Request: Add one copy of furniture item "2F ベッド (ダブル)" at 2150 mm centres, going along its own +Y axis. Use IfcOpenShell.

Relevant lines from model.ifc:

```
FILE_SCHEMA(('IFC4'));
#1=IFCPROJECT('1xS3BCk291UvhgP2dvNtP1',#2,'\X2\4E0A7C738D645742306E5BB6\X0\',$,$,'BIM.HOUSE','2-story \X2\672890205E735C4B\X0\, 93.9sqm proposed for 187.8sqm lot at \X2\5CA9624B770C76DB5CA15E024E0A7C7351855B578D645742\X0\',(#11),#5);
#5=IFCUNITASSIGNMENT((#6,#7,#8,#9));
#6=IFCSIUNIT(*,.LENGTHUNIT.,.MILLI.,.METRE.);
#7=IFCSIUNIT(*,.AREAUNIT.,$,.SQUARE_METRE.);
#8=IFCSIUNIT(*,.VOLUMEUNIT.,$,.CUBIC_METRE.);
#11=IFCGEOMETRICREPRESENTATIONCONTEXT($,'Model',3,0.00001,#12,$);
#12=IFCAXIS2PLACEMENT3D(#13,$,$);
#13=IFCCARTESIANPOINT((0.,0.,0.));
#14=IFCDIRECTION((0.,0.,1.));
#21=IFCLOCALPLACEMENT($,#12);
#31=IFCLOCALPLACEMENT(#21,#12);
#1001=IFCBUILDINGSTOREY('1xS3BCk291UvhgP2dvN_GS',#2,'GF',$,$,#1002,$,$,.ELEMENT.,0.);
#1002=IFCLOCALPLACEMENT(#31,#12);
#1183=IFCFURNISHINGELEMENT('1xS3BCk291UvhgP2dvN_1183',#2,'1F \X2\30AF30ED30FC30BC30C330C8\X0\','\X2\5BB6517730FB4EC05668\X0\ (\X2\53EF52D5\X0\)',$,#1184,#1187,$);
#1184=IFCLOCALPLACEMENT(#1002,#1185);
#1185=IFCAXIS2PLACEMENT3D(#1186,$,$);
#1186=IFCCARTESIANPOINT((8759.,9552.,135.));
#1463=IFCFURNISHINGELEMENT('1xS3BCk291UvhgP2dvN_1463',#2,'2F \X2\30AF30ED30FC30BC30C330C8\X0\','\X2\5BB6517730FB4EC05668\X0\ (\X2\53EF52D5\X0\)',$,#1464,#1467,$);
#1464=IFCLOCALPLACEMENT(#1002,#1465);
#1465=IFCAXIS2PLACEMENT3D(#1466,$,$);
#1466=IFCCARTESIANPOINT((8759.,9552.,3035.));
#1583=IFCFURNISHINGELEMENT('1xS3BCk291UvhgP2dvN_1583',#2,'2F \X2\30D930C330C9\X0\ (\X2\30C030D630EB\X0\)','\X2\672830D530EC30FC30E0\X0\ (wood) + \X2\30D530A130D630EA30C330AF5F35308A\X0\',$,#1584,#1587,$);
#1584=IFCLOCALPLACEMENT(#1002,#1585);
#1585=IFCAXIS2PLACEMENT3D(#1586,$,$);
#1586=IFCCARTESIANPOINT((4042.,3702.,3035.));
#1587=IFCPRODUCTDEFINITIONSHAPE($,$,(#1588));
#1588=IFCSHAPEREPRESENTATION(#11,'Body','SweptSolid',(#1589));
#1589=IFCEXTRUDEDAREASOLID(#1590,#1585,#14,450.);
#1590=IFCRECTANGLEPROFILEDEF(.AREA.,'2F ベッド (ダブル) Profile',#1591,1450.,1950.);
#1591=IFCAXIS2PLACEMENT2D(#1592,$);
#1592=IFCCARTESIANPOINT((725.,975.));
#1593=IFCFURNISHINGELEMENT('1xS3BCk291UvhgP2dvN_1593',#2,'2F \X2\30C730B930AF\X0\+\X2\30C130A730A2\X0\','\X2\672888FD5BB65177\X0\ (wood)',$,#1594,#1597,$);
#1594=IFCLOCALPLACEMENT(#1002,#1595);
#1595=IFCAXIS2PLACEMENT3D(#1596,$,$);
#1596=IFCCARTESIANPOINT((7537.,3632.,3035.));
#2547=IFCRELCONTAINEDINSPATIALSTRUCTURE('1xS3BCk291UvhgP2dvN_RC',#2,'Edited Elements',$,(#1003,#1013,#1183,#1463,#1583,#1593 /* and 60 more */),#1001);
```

```python
import ifcopenshell
import ifcopenshell.api.geometry
import ifcopenshell.api.root
import ifcopenshell.util.element
import ifcopenshell.util.placement
import ifcopenshell.util.unit

model = ifcopenshell.open("model.ifc")
unit_scale = ifcopenshell.util.unit.calculate_unit_scale(model)


def reuse_history(source, copy):
    """copy_class also copies each property set's owner history, people and application; keep the originals."""
    for rel in copy.IsDefinedBy:
        if rel.is_a("IfcRelDefinesByProperties") and (history := rel.RelatingPropertyDefinition.OwnerHistory):
            rel.RelatingPropertyDefinition.OwnerHistory = source.OwnerHistory
            ifcopenshell.util.element.remove_deep2(model, history)


source = model.by_id(1583)
base = ifcopenshell.util.placement.get_local_placement(source.ObjectPlacement)
step = base[:3, 1] * 2.15 / unit_scale

for i in range(1, 2):
    copy = ifcopenshell.api.root.copy_class(model, product=source)
    copy.Representation = ifcopenshell.util.element.copy_deep(
        model, source.Representation, exclude=["IfcGeometricRepresentationContext", "IfcRepresentationMap"]
    )
    reuse_history(source, copy)
    matrix = base.copy()
    matrix[:3, 3] += i * step
    print("added at", matrix[:3, 3].round(3) + 0.0)
    ifcopenshell.api.geometry.edit_object_placement(model, product=copy, matrix=matrix, is_si=False)

model.write("model_rev.ifc")
```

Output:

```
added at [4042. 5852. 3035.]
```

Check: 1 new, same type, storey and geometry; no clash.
